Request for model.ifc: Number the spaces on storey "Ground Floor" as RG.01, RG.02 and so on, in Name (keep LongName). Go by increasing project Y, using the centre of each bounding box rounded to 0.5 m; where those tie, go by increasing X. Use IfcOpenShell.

First a look at what the model holds.

```python
import ifcopenshell
import ifcopenshell.util.element
import ifcopenshell.util.placement

model = ifcopenshell.open("model.ifc")
print(model.schema)
storey = next(s for s in model.by_type("IfcBuildingStorey") if s.Name == "Ground Floor")
spaces = [e for e in ifcopenshell.util.element.get_decomposition(storey) if e.is_a("IfcSpace")]
for e in sorted(spaces, key=lambda e: e.id()):
    origin = ifcopenshell.util.placement.get_local_placement(e.ObjectPlacement)[:3, 3]
    print(e.id(), e.Name, e.LongName, origin.round(2) + 0.0, sep=" | ")
```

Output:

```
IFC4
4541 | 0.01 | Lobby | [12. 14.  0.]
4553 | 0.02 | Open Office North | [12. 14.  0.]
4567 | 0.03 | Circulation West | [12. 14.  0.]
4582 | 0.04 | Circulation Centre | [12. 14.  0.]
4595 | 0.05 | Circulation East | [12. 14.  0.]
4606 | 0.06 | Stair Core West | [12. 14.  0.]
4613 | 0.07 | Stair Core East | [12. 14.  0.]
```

```python
import ifcopenshell
import ifcopenshell.geom
import ifcopenshell.util.element
import ifcopenshell.util.shape

model = ifcopenshell.open("model.ifc")
settings = ifcopenshell.geom.settings()
settings.set("use-world-coords", True)


def centre(element):
    shape = ifcopenshell.geom.create_shape(settings, element)
    return ifcopenshell.util.shape.get_bbox_centroid(shape.geometry)


storey = next(s for s in model.by_type("IfcBuildingStorey") if s.Name == "Ground Floor")
spaces = [e for e in ifcopenshell.util.element.get_decomposition(storey) if e.is_a("IfcSpace")]

# Insertion points can sit at a corner or the storey origin, so sort by the geometry (in metres).
centres = {e: centre(e) for e in spaces}
spaces.sort(key=lambda e: (round(centres[e][1] / 0.5), centres[e][0]))

for i, e in enumerate(spaces, start=1):
    number = f"RG.{i:02d}"
    e.Name = number
    print(e.id(), number)

model.write("model_rev.ifc")
```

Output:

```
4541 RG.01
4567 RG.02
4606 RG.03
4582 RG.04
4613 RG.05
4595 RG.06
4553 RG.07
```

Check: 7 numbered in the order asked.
